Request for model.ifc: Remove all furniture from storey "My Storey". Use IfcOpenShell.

First a look at what the model holds.

```python
import ifcopenshell
import ifcopenshell.util.element

model = ifcopenshell.open("model.ifc")
print(model.schema)
storey = next(s for s in model.by_type("IfcBuildingStorey") if s.Name == "My Storey")
furniture = [e for e in ifcopenshell.util.element.get_decomposition(storey) if e.is_a("IfcFurnishingElement")]
seen = {}
for e in furniture:
    element_type = ifcopenshell.util.element.get_type(e)
    name = element_type.Name if element_type not in (None, e) else None
    seen[name] = seen.get(name, 0) + 1
for name, count in sorted(seen.items(), key=str):
    print(count, "x", name)
```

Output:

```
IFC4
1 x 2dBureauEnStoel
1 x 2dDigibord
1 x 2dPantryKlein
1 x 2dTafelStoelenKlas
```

```python
import ifcopenshell
import ifcopenshell.api.root
import ifcopenshell.util.element

model = ifcopenshell.open("model.ifc")

storey = next(s for s in model.by_type("IfcBuildingStorey") if s.Name == "My Storey")
furniture = [e for e in ifcopenshell.util.element.get_decomposition(storey) if e.is_a("IfcFurnishingElement")]

for e in furniture:
    ifcopenshell.api.root.remove_product(model, product=e)
print(len(furniture), "removed")

model.write("model_rev.ifc")
```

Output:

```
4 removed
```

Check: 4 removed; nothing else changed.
